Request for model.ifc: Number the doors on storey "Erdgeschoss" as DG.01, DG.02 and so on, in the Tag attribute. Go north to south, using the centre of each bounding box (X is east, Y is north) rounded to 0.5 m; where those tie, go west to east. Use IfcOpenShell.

First a look at what the model holds.

```python
import ifcopenshell
import ifcopenshell.util.element
import ifcopenshell.util.placement

model = ifcopenshell.open("model.ifc")
print(model.schema)
storey = next(s for s in model.by_type("IfcBuildingStorey") if s.Name == "Erdgeschoss")
doors = [e for e in ifcopenshell.util.element.get_decomposition(storey) if e.is_a("IfcDoor")]
for e in sorted(doors, key=lambda e: e.id()):
    origin = ifcopenshell.util.placement.get_local_placement(e.ObjectPlacement)[:3, 3]
    print(e.id(), e.Tag, e.Name, origin.round(2) + 0.0, sep=" | ")
```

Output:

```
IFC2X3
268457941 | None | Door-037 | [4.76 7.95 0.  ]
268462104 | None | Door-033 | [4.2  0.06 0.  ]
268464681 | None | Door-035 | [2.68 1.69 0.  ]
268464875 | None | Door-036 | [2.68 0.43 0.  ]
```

```python
import ifcopenshell
import ifcopenshell.geom
import ifcopenshell.util.element
import ifcopenshell.util.shape

model = ifcopenshell.open("model.ifc")
settings = ifcopenshell.geom.settings()
settings.set("use-world-coords", True)


def centre(element):
    shape = ifcopenshell.geom.create_shape(settings, element)
    return ifcopenshell.util.shape.get_bbox_centroid(shape.geometry)


storey = next(s for s in model.by_type("IfcBuildingStorey") if s.Name == "Erdgeschoss")
doors = [e for e in ifcopenshell.util.element.get_decomposition(storey) if e.is_a("IfcDoor")]

# Insertion points can sit at a corner or the storey origin, so sort by the geometry (in metres).
centres = {e: centre(e) for e in doors}
doors.sort(key=lambda e: (-round(centres[e][1] / 0.5), centres[e][0]))

for i, e in enumerate(doors, start=1):
    number = f"DG.{i:02d}"
    e.Tag = number
    print(e.id(), number)

model.write("model-out.ifc")
```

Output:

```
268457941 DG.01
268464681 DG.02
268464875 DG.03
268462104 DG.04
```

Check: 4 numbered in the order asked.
